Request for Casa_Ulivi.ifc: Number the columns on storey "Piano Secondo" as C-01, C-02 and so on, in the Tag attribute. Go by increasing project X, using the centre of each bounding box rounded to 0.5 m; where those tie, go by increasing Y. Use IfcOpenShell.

First a look at what the model holds.

```python
import ifcopenshell
import ifcopenshell.util.element
import ifcopenshell.util.placement

model = ifcopenshell.open("Casa_Ulivi.ifc")
print(model.schema)
storey = next(s for s in model.by_type("IfcBuildingStorey") if s.Name == "Piano Secondo")
columns = [e for e in ifcopenshell.util.element.get_decomposition(storey) if e.is_a("IfcColumn")]
for e in sorted(columns, key=lambda e: e.id()):
    origin = ifcopenshell.util.placement.get_local_placement(e.ObjectPlacement)[:3, 3]
    print(e.id(), e.Tag, e.Name, origin.round(2) + 0.0, sep=" | ")
```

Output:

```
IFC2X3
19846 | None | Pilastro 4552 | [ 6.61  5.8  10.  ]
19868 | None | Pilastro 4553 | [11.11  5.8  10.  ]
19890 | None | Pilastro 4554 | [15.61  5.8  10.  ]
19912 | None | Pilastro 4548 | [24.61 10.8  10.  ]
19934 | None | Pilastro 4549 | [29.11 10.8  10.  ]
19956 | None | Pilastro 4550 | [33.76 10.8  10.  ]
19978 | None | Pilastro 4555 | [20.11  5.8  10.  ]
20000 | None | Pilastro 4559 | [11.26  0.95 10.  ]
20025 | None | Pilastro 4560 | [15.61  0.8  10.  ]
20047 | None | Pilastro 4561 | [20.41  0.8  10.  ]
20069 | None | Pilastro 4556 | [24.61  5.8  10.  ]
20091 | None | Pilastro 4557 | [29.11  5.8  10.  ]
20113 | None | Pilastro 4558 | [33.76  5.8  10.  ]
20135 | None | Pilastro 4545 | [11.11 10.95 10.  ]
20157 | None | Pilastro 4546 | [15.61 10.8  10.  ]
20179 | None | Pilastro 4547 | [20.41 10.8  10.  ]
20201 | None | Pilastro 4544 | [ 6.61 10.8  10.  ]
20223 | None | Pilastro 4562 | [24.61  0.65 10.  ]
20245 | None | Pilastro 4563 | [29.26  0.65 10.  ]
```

```python
import ifcopenshell
import ifcopenshell.geom
import ifcopenshell.util.element
import ifcopenshell.util.shape

model = ifcopenshell.open("Casa_Ulivi.ifc")
settings = ifcopenshell.geom.settings()
settings.set("use-world-coords", True)


def centre(element):
    shape = ifcopenshell.geom.create_shape(settings, element)
    return ifcopenshell.util.shape.get_bbox_centroid(shape.geometry)


storey = next(s for s in model.by_type("IfcBuildingStorey") if s.Name == "Piano Secondo")
columns = [e for e in ifcopenshell.util.element.get_decomposition(storey) if e.is_a("IfcColumn")]

# Insertion points can sit at a corner or the storey origin, so sort by the geometry (in metres).
centres = {e: centre(e) for e in columns}
columns.sort(key=lambda e: (round(centres[e][0] / 0.5), centres[e][1]))

for i, e in enumerate(columns, start=1):
    number = f"C-{i:02d}"
    e.Tag = number
    print(e.id(), number)

model.write("Casa_Ulivi_rev.ifc")
```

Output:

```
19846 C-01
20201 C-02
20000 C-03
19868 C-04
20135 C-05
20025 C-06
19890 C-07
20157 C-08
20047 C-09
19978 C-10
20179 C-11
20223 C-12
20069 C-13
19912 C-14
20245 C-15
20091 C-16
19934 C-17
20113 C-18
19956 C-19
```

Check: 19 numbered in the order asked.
